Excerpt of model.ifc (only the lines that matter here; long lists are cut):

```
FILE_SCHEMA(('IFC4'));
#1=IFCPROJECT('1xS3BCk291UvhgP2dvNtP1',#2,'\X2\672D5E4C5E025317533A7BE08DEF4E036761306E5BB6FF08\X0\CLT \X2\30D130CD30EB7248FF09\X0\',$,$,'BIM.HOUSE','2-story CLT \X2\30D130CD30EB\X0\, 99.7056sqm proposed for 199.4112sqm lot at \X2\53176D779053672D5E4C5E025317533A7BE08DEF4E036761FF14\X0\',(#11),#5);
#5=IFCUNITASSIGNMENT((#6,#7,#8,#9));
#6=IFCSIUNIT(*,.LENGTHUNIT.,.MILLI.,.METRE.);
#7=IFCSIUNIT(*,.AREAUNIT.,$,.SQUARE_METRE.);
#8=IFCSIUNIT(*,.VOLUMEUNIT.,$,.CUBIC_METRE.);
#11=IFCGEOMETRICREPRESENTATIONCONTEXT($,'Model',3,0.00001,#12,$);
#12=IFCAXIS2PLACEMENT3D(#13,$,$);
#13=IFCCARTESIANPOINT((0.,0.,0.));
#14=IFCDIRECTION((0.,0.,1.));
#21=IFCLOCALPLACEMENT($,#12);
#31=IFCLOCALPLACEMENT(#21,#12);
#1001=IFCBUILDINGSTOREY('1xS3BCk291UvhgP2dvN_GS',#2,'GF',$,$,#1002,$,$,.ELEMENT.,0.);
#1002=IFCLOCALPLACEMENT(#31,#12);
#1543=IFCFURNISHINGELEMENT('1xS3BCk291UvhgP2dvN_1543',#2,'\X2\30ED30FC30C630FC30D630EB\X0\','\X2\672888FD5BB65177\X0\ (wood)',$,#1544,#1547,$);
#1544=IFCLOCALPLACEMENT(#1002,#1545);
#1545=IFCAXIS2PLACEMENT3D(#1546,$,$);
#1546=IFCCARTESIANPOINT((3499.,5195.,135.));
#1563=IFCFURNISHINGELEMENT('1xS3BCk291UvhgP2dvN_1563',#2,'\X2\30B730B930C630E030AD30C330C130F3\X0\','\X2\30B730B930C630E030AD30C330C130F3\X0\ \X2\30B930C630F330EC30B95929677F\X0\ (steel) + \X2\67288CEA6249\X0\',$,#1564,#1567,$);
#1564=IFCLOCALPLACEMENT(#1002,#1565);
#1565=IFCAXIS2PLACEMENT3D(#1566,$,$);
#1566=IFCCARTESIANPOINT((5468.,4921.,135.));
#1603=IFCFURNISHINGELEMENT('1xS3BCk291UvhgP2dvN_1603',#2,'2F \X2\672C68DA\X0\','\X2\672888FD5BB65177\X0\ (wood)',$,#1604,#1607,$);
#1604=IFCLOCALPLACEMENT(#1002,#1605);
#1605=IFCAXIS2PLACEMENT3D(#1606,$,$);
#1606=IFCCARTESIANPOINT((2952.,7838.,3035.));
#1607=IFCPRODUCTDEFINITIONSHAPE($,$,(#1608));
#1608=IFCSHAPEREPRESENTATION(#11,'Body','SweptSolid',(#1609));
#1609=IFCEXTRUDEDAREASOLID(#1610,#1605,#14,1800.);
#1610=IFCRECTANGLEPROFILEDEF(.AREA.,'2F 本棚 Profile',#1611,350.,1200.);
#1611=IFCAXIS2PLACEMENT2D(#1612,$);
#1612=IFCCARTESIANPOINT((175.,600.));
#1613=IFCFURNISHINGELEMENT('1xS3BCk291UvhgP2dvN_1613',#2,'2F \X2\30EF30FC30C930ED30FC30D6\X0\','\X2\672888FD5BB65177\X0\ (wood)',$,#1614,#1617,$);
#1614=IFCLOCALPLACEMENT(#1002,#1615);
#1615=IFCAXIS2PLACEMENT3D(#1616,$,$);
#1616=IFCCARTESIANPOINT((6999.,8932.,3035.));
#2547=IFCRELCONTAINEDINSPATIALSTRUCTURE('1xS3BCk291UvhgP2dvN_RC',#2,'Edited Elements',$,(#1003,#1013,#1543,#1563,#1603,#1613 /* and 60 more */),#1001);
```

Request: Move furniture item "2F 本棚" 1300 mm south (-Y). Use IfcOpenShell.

```python
import ifcopenshell
import ifcopenshell.api.geometry
import ifcopenshell.util.placement
import ifcopenshell.util.unit

model = ifcopenshell.open("model.ifc")
unit_scale = ifcopenshell.util.unit.calculate_unit_scale(model)

item = model.by_id(1603)
matrix = ifcopenshell.util.placement.get_local_placement(item.ObjectPlacement)
matrix[1, 3] -= 1.3 / unit_scale
ifcopenshell.api.geometry.edit_object_placement(model, product=item, matrix=matrix, is_si=False)

print(ifcopenshell.util.placement.get_local_placement(item.ObjectPlacement).round(3) + 0.0)

model.write("model_edited.ifc")
```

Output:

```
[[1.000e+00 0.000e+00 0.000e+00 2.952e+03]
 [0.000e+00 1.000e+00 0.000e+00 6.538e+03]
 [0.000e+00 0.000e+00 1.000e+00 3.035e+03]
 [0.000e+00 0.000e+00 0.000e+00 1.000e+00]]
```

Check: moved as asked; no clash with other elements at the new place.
